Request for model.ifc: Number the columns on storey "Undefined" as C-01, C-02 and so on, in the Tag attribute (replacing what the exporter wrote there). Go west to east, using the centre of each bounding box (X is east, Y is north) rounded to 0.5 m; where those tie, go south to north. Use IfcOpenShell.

First a look at what the model holds.

```python
import ifcopenshell
import ifcopenshell.util.element
import ifcopenshell.util.placement

model = ifcopenshell.open("model.ifc")
print(model.schema)
storey = next(s for s in model.by_type("IfcBuildingStorey") if s.Name == "Undefined")
columns = [e for e in ifcopenshell.util.element.get_decomposition(storey) if e.is_a("IfcColumn")]
for e in sorted(columns, key=lambda e: e.id()):
    origin = ifcopenshell.util.placement.get_local_placement(e.ObjectPlacement)[:3, 3]
    print(e.id(), e.Tag, e.Name, origin.round(2) + 0.0, sep=" | ")
```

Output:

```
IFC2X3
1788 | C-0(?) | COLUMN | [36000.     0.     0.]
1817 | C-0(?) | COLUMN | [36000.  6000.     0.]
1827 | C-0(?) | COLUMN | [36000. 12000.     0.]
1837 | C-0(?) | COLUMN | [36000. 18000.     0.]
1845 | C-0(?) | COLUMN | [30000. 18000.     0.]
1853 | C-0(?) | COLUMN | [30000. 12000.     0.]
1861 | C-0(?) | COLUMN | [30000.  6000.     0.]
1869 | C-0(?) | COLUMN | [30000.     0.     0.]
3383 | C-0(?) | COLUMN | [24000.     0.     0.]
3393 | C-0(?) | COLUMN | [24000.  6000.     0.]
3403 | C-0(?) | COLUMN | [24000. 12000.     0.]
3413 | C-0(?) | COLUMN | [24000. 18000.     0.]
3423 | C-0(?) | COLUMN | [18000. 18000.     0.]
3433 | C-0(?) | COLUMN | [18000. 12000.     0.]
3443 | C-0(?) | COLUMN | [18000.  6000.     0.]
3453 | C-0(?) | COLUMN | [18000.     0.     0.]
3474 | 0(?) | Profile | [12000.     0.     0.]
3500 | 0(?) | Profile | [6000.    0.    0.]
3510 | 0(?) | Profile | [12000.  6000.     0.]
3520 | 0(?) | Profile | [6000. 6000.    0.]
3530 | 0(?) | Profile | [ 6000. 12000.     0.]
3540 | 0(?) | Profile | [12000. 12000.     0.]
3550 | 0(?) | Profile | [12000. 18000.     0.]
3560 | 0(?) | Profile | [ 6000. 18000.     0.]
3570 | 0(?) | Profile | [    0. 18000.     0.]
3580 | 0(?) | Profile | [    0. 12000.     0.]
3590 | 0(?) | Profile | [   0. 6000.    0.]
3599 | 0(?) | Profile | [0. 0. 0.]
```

```python
import ifcopenshell
import ifcopenshell.geom
import ifcopenshell.util.element
import ifcopenshell.util.shape

model = ifcopenshell.open("model.ifc")
settings = ifcopenshell.geom.settings()
settings.set("use-world-coords", True)


def centre(element):
    shape = ifcopenshell.geom.create_shape(settings, element)
    return ifcopenshell.util.shape.get_bbox_centroid(shape.geometry)


storey = next(s for s in model.by_type("IfcBuildingStorey") if s.Name == "Undefined")
columns = [e for e in ifcopenshell.util.element.get_decomposition(storey) if e.is_a("IfcColumn")]

# Insertion points can sit at a corner or the storey origin, so sort by the geometry (in metres).
centres = {e: centre(e) for e in columns}
columns.sort(key=lambda e: (round(centres[e][0] / 0.5), centres[e][1]))

for i, e in enumerate(columns, start=1):
    number = f"C-{i:02d}"
    e.Tag = number
    print(e.id(), number)

model.write("model_edited.ifc")
```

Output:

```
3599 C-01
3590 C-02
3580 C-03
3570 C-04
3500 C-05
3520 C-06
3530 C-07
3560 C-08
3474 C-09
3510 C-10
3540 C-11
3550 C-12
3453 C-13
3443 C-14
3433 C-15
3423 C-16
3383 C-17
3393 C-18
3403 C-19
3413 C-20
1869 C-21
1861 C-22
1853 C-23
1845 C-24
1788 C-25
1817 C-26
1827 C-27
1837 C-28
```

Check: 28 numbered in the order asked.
